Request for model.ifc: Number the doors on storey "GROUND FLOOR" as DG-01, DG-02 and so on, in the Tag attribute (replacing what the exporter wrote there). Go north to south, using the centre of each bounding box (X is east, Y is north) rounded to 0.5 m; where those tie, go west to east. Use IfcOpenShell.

First a look at what the model holds.

```python
import ifcopenshell
import ifcopenshell.util.element
import ifcopenshell.util.placement

model = ifcopenshell.open("model.ifc")
print(model.schema)
storey = next(s for s in model.by_type("IfcBuildingStorey") if s.Name == "GROUND FLOOR")
doors = [e for e in ifcopenshell.util.element.get_decomposition(storey) if e.is_a("IfcDoor")]
for e in sorted(doors, key=lambda e: e.id()):
    origin = ifcopenshell.util.placement.get_local_placement(e.ObjectPlacement)[:3, 3]
    print(e.id(), e.Tag, e.Name, origin.round(2) + 0.0, sep=" | ")
```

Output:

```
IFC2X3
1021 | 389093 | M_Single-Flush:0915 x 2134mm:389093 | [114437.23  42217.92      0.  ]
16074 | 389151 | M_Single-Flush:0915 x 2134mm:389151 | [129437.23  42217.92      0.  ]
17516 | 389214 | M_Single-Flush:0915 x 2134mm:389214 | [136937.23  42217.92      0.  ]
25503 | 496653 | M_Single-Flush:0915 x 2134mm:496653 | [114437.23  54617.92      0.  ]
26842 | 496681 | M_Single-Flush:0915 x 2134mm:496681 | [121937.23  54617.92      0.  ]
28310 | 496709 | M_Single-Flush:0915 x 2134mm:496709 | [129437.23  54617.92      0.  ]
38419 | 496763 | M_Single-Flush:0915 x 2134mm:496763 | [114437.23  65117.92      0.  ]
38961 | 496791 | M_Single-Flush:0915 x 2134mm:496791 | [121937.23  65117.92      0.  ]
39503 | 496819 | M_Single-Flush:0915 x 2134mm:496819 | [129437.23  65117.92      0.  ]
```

```python
import ifcopenshell
import ifcopenshell.geom
import ifcopenshell.util.element
import ifcopenshell.util.shape

model = ifcopenshell.open("model.ifc")
settings = ifcopenshell.geom.settings()
settings.set("use-world-coords", True)


def centre(element):
    shape = ifcopenshell.geom.create_shape(settings, element)
    return ifcopenshell.util.shape.get_bbox_centroid(shape.geometry)


storey = next(s for s in model.by_type("IfcBuildingStorey") if s.Name == "GROUND FLOOR")
doors = [e for e in ifcopenshell.util.element.get_decomposition(storey) if e.is_a("IfcDoor")]

# Insertion points can sit at a corner or the storey origin, so sort by the geometry (in metres).
centres = {e: centre(e) for e in doors}
doors.sort(key=lambda e: (-round(centres[e][1] / 0.5), centres[e][0]))

for i, e in enumerate(doors, start=1):
    number = f"DG-{i:02d}"
    e.Tag = number
    print(e.id(), number)

model.write("model_updated.ifc")
```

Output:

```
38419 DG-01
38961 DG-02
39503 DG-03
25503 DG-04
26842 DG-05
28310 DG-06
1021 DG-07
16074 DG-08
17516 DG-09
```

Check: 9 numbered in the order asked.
